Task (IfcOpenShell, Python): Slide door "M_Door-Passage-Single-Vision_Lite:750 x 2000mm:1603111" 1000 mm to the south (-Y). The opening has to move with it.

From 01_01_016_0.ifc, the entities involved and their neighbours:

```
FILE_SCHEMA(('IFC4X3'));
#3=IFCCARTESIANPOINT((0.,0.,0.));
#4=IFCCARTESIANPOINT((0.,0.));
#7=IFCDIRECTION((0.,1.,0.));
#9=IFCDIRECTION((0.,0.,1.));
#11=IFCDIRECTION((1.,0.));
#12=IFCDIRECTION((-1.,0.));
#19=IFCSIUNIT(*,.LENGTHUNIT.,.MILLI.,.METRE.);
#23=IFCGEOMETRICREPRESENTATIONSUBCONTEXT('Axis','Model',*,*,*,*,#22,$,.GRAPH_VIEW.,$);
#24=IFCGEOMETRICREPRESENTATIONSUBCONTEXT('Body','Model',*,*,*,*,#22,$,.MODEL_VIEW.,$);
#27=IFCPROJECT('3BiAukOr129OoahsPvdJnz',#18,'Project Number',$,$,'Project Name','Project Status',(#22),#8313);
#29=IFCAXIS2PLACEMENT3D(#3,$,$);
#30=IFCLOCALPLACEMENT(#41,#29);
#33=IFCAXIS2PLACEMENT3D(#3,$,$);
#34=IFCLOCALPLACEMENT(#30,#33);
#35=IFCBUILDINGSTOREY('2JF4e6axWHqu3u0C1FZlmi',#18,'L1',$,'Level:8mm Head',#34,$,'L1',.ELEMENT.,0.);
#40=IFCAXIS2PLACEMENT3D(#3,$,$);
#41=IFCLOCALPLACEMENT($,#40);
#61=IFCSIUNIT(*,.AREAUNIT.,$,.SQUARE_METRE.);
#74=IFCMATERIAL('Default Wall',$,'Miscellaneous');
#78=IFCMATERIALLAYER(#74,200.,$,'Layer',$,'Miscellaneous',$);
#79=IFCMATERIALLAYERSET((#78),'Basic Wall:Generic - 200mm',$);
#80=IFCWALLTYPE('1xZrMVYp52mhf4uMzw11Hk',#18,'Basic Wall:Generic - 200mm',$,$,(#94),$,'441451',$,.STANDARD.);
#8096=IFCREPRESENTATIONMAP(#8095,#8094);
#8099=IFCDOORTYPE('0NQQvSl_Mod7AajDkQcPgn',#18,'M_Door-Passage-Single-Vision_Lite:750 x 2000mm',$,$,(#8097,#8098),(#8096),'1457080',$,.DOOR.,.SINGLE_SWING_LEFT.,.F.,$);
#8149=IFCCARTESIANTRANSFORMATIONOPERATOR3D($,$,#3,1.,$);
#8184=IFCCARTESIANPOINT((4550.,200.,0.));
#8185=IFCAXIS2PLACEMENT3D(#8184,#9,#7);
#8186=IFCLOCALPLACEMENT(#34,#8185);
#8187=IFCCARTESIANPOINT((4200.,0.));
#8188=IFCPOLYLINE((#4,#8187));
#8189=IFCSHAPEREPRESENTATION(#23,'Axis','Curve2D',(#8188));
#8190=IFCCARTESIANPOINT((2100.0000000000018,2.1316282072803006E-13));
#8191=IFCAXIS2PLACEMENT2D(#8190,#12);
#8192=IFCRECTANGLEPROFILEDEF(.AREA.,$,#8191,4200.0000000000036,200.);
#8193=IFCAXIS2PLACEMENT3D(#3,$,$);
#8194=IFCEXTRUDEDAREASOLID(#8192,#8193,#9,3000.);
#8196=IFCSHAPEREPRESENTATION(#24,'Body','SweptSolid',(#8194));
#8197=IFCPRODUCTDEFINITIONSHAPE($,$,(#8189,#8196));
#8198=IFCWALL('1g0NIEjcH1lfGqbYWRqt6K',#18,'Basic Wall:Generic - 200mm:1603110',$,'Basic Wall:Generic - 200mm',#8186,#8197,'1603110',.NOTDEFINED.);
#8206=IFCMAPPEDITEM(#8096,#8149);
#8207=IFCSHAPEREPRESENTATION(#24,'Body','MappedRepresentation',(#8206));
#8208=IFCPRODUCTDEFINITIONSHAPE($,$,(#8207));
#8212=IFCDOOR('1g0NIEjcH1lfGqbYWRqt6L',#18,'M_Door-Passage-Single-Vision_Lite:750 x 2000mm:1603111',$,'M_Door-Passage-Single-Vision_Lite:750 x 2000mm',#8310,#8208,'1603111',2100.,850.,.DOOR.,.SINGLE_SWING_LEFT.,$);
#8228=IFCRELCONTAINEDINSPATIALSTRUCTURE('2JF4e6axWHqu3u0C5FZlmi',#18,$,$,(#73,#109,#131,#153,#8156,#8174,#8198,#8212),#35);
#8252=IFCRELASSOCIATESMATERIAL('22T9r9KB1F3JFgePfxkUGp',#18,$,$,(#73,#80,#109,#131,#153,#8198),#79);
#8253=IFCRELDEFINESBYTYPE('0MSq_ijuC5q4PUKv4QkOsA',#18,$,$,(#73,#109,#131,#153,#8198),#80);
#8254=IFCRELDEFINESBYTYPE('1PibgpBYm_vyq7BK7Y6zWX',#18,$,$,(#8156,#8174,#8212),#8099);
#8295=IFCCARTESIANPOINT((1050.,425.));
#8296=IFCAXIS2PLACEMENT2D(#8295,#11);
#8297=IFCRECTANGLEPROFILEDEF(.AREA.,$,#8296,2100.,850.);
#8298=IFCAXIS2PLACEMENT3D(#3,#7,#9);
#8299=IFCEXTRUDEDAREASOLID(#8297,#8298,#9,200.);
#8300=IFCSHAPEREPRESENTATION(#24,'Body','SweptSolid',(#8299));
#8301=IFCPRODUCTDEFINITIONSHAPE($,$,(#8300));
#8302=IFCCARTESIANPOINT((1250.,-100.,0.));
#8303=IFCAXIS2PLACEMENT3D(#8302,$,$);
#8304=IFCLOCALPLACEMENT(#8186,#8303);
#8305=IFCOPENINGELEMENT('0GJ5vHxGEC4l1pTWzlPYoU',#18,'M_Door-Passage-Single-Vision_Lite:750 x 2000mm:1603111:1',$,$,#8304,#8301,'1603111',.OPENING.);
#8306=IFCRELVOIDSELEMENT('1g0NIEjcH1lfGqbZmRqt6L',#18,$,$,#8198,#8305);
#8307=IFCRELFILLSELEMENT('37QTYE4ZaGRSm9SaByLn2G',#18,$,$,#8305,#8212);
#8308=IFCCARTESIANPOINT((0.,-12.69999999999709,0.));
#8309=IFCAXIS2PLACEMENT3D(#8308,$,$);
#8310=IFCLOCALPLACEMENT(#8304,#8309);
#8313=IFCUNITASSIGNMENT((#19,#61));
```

```python
import ifcopenshell
import ifcopenshell.api.geometry
import ifcopenshell.util.placement
import ifcopenshell.util.unit

model = ifcopenshell.open("01_01_016_0.ifc")
unit_scale = ifcopenshell.util.unit.calculate_unit_scale(model)

door = model.by_guid("1g0NIEjcH1lfGqbYWRqt6L")
opening = door.FillsVoids[0].RelatingOpeningElement
wall = opening.VoidsElements[0].RelatingBuildingElement

wall_matrix = ifcopenshell.util.placement.get_local_placement(wall.ObjectPlacement)
shift = wall_matrix[:3, 0] * -1 / unit_scale
before = ifcopenshell.util.placement.get_local_placement(door.ObjectPlacement)[:3, 3].copy()

# The door is placed relative to its opening, so it follows when the opening moves.
matrix = ifcopenshell.util.placement.get_local_placement(opening.ObjectPlacement)
matrix[:3, 3] += shift
ifcopenshell.api.geometry.edit_object_placement(
    model, product=opening, matrix=matrix, is_si=False, should_transform_children=True
)

after = ifcopenshell.util.placement.get_local_placement(door.ObjectPlacement)[:3, 3]
print("door moved by", (after - before).round(3) + 0.0)

model.write("01_01_016_0-out.ifc")
```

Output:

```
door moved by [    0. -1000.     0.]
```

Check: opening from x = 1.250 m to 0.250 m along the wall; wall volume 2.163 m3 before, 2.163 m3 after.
